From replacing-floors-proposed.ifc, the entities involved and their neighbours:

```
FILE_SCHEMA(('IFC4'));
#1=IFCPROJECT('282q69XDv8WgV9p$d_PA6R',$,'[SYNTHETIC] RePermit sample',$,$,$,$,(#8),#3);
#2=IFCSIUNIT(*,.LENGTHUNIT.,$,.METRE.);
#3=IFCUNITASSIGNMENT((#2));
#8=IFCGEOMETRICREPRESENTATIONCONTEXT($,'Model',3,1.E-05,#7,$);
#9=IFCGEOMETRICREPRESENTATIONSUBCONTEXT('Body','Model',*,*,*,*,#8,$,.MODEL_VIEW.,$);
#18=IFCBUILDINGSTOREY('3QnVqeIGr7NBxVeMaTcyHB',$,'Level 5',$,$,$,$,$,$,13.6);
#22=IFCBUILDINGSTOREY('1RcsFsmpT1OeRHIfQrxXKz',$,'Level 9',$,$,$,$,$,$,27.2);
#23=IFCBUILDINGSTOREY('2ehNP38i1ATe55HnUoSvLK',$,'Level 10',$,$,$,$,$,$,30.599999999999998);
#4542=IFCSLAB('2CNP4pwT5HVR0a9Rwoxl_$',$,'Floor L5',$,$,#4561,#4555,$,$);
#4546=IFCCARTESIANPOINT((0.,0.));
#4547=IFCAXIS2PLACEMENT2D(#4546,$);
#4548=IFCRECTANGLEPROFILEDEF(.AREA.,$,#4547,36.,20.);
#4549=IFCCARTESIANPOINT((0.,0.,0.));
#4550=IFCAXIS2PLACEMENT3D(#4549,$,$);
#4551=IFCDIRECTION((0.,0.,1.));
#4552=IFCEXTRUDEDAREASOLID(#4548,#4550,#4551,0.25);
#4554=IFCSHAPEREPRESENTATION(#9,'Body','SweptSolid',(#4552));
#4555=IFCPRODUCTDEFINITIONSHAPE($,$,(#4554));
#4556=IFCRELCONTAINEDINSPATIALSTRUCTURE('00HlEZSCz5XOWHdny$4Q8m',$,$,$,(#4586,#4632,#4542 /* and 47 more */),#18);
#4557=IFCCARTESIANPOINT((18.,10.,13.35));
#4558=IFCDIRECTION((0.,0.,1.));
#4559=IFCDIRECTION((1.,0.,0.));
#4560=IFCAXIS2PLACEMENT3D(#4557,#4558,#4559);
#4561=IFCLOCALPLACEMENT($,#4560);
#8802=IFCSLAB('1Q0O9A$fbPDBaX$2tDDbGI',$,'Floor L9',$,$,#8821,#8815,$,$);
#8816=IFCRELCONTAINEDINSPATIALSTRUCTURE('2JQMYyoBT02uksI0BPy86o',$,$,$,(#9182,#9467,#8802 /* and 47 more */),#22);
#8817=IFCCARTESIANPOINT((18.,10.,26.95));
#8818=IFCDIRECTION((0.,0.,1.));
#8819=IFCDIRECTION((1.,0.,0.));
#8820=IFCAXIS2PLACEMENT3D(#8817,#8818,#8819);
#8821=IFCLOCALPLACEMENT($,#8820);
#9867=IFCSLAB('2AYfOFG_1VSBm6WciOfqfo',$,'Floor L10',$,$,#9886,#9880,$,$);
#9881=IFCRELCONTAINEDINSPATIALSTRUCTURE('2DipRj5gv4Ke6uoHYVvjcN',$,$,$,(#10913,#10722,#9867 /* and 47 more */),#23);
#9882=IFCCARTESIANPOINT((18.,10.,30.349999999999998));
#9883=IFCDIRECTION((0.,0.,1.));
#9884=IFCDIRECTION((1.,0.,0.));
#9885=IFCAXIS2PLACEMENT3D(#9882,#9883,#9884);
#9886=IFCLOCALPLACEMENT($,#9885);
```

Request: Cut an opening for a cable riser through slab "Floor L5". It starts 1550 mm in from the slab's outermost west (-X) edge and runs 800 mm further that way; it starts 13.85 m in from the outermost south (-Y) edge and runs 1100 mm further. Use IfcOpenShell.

```python
import numpy as np
import ifcopenshell
import ifcopenshell.api.feature
import ifcopenshell.api.geometry
import ifcopenshell.api.root
import ifcopenshell.geom
import ifcopenshell.util.placement
import ifcopenshell.util.representation
import ifcopenshell.util.shape
import ifcopenshell.util.unit

model = ifcopenshell.open("replacing-floors-proposed.ifc")
unit_scale = ifcopenshell.util.unit.calculate_unit_scale(model)
settings = ifcopenshell.geom.settings()


def volume(element):
    """Net volume in cubic metres, openings subtracted."""
    shape = ifcopenshell.geom.create_shape(settings, element)
    return ifcopenshell.util.shape.get_volume(shape.geometry)


slab = model.by_id(4542)
before = volume(slab)

# Extent in the slab's own axes, in metres. The edges named are its -X and -Y sides.
slab_shape = ifcopenshell.geom.create_shape(settings, slab)
vertices = ifcopenshell.util.shape.get_vertices(slab_shape.geometry)
x_min, y_min, bottom = vertices.min(axis=0)
top = vertices[:, 2].max()

opening = ifcopenshell.api.root.create_entity(model, ifc_class="IfcOpeningElement", name="Cable riser opening", predefined_type="OPENING")
context = ifcopenshell.util.representation.get_context(model, "Model", "Body", "MODEL_VIEW")
width, depth = 0.8, 1.1
outline = [(0.0, 0.0), (width, 0.0), (width, depth), (0.0, depth), (0.0, 0.0)]
# Overshoot both faces by 50 mm so the cut is clean.
shape = ifcopenshell.api.geometry.add_slab_representation(
    model, context=context, depth=top - bottom + 0.1, polyline=outline
)
ifcopenshell.api.geometry.assign_representation(model, product=opening, representation=shape)

matrix = ifcopenshell.util.placement.get_local_placement(slab.ObjectPlacement)
matrix[:, 3] = matrix @ np.append(np.array([x_min + 1.55, y_min + 13.85, bottom - 0.05]) / unit_scale, 1.0)
ifcopenshell.api.geometry.edit_object_placement(model, product=opening, matrix=matrix, is_si=False)
ifcopenshell.api.feature.add_feature(model, feature=opening, element=slab)

after = volume(slab)

print(f"slab volume {before:.3f} -> {after:.3f} m3")

model.write("replacing-floors-proposed-out.ifc")
```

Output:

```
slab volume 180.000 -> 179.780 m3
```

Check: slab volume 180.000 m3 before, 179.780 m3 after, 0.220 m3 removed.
